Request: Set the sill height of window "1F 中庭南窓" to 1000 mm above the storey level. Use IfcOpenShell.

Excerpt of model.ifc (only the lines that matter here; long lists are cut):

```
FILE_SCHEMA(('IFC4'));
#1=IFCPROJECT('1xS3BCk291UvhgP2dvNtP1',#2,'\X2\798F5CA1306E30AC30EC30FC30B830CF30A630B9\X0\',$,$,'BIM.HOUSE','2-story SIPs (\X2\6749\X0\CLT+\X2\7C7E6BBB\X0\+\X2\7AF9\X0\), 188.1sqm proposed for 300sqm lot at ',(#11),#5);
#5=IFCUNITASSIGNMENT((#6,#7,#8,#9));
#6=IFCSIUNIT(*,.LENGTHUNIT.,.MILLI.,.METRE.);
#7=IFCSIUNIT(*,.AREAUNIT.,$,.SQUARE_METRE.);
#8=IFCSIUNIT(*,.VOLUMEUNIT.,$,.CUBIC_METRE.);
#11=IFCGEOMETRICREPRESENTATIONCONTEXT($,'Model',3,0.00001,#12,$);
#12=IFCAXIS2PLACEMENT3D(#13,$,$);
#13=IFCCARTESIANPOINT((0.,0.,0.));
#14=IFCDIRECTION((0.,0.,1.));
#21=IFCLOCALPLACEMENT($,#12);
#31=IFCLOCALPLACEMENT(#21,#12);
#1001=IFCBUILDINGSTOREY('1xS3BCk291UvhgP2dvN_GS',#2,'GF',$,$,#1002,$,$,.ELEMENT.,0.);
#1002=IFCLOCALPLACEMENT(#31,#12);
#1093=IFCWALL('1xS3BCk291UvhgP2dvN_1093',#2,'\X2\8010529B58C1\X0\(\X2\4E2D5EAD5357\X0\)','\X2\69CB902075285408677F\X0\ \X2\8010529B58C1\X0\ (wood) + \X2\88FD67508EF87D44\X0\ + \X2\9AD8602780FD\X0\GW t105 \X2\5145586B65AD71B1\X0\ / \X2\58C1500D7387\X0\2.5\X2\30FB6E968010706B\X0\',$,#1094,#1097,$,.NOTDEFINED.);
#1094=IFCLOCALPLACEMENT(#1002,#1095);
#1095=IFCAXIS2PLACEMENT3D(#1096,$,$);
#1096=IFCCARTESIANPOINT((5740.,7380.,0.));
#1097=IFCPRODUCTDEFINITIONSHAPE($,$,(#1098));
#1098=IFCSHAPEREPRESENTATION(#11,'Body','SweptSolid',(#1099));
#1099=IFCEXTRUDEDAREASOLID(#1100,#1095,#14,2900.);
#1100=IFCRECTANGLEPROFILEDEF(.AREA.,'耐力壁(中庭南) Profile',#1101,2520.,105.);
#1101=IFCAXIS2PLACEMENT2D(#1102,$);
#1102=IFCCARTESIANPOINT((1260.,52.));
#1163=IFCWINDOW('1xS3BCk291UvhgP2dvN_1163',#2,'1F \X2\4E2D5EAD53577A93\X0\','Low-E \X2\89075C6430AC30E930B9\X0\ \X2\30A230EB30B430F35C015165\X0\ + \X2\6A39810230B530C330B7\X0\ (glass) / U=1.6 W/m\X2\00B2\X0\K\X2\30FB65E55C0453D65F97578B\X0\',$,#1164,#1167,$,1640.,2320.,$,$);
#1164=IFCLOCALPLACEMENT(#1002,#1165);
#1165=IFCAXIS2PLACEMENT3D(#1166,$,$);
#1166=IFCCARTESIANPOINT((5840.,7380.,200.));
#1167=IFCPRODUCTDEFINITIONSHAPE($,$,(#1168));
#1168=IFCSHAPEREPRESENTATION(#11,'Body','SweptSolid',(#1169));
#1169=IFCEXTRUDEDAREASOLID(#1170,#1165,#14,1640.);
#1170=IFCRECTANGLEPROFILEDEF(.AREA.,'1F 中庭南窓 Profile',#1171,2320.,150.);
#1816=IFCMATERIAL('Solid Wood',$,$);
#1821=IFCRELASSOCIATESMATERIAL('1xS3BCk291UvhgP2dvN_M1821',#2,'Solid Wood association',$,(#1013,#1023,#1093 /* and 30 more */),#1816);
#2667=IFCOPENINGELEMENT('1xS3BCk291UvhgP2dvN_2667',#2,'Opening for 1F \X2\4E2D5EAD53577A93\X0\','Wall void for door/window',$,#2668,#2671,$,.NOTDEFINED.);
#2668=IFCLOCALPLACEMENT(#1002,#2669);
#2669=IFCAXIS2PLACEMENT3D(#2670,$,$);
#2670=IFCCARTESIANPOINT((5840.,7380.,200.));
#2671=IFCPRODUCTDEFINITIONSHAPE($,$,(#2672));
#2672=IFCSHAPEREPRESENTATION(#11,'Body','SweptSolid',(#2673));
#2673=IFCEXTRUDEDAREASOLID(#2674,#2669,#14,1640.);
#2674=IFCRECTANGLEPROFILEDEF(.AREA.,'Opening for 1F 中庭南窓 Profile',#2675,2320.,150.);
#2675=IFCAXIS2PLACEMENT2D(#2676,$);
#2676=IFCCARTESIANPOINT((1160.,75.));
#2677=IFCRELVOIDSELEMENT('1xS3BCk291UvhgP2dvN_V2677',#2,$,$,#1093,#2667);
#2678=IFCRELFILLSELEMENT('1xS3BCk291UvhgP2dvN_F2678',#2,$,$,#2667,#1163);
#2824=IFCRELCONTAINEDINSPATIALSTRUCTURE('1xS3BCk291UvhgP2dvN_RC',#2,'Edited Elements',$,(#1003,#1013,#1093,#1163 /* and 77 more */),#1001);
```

```python
import numpy as np
import ifcopenshell
import ifcopenshell.api.geometry
import ifcopenshell.geom
import ifcopenshell.util.element
import ifcopenshell.util.placement
import ifcopenshell.util.shape
import ifcopenshell.util.unit

model = ifcopenshell.open("model.ifc")
unit_scale = ifcopenshell.util.unit.calculate_unit_scale(model)

window = model.by_id(1163)
opening = window.FillsVoids[0].RelatingOpeningElement
storey = ifcopenshell.util.element.get_container(window, ifc_class="IfcBuildingStorey")
level = ifcopenshell.util.placement.get_local_placement(storey.ObjectPlacement)[2, 3]

# The opening's origin need not be at the sill, so measure its lowest point.
shape = ifcopenshell.geom.create_shape(ifcopenshell.geom.settings(), opening)
bottom = ifcopenshell.util.shape.get_shape_bottom_elevation(shape, shape.geometry) / unit_scale
dz = level + 1 / unit_scale - bottom

shift = np.array([0.0, 0.0, dz])
# The window is not placed relative to its opening, so move both.
for product in (opening, window):
    matrix = ifcopenshell.util.placement.get_local_placement(product.ObjectPlacement)
    matrix[:3, 3] += shift
    ifcopenshell.api.geometry.edit_object_placement(model, product=product, matrix=matrix, is_si=False)

print(f"moved by {dz * unit_scale:+.3f} m")

model.write("model_updated.ifc")
```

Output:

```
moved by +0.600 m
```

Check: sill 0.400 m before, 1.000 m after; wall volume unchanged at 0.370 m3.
